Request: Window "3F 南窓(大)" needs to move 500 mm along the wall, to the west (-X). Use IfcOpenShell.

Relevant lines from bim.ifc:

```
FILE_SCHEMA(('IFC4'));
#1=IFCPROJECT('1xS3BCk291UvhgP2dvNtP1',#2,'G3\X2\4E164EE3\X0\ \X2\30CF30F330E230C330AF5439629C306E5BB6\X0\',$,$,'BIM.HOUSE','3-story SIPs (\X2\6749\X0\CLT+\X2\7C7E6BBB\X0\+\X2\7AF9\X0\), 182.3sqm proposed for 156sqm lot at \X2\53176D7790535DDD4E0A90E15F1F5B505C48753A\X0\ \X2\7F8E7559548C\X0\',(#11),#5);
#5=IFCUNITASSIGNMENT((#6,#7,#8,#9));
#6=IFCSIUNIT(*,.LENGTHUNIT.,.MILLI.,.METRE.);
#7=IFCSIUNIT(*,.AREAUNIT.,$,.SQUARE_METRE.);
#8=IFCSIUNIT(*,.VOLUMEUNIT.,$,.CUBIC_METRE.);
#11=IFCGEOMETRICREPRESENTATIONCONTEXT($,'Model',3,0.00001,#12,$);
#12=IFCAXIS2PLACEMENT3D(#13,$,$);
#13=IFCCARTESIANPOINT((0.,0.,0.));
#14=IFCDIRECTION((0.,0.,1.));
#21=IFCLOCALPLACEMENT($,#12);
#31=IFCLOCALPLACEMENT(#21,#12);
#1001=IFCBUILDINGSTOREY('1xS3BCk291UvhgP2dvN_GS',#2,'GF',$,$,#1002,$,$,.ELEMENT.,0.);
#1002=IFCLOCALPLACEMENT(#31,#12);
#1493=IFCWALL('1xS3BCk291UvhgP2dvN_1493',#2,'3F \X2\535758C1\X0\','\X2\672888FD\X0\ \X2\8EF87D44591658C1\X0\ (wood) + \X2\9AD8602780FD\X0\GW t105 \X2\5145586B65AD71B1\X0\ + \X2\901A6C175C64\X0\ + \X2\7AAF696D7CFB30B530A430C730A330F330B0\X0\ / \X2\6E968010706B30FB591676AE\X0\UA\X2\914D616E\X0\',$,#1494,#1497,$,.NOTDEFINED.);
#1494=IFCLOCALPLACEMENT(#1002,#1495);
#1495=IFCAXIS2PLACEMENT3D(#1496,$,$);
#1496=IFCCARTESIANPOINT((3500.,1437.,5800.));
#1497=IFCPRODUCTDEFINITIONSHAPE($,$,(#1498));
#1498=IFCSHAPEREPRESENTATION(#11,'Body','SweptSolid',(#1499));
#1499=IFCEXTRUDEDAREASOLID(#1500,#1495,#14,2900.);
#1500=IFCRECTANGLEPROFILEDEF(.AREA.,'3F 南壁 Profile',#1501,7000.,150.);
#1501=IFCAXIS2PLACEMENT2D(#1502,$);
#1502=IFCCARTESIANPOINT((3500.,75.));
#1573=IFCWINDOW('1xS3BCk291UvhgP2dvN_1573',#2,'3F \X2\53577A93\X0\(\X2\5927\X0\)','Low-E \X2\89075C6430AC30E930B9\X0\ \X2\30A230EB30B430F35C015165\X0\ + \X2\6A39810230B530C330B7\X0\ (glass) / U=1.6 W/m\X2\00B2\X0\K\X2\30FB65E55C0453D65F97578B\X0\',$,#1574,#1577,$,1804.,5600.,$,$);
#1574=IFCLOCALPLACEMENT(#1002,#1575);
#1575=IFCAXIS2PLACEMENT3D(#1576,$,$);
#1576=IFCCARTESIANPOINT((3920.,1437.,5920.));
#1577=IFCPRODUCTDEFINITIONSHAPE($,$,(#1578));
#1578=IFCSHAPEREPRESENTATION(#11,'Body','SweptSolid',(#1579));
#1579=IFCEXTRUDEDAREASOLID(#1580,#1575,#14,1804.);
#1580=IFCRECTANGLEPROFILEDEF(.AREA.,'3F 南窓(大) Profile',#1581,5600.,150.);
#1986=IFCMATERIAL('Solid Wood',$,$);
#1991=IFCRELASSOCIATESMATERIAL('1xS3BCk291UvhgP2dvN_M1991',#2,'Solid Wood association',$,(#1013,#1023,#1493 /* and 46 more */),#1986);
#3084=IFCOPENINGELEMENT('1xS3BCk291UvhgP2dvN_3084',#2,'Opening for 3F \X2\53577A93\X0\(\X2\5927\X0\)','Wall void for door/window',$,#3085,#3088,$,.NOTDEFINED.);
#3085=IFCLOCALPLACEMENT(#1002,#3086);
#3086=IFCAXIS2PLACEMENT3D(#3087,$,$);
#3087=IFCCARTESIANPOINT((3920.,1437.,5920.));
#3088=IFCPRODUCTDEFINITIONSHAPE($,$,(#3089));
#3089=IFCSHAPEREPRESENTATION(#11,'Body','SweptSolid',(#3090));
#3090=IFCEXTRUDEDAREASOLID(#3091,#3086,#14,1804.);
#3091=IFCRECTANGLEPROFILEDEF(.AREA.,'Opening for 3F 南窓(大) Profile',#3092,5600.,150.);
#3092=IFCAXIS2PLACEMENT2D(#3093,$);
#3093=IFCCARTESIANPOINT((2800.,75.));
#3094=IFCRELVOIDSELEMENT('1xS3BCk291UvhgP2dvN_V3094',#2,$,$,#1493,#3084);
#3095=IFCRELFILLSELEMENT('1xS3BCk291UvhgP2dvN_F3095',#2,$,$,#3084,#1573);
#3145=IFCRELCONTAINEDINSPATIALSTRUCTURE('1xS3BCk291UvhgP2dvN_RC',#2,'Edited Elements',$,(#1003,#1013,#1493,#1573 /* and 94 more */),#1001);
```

```python
import ifcopenshell
import ifcopenshell.api.geometry
import ifcopenshell.util.placement
import ifcopenshell.util.unit

model = ifcopenshell.open("bim.ifc")
unit_scale = ifcopenshell.util.unit.calculate_unit_scale(model)

window = model.by_id(1573)
opening = window.FillsVoids[0].RelatingOpeningElement
wall = opening.VoidsElements[0].RelatingBuildingElement

wall_matrix = ifcopenshell.util.placement.get_local_placement(wall.ObjectPlacement)
shift = wall_matrix[:3, 0] * -0.5 / unit_scale
before = ifcopenshell.util.placement.get_local_placement(window.ObjectPlacement)[:3, 3].copy()

# The window is not placed relative to its opening, so move both.
for product in (opening, window):
    matrix = ifcopenshell.util.placement.get_local_placement(product.ObjectPlacement)
    matrix[:3, 3] += shift
    ifcopenshell.api.geometry.edit_object_placement(model, product=product, matrix=matrix, is_si=False)

after = ifcopenshell.util.placement.get_local_placement(window.ObjectPlacement)[:3, 3]
print("window moved by", (after - before).round(3) + 0.0)

model.write("bim_rev.ifc")
```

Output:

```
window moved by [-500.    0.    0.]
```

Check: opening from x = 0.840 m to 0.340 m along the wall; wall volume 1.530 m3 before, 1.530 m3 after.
